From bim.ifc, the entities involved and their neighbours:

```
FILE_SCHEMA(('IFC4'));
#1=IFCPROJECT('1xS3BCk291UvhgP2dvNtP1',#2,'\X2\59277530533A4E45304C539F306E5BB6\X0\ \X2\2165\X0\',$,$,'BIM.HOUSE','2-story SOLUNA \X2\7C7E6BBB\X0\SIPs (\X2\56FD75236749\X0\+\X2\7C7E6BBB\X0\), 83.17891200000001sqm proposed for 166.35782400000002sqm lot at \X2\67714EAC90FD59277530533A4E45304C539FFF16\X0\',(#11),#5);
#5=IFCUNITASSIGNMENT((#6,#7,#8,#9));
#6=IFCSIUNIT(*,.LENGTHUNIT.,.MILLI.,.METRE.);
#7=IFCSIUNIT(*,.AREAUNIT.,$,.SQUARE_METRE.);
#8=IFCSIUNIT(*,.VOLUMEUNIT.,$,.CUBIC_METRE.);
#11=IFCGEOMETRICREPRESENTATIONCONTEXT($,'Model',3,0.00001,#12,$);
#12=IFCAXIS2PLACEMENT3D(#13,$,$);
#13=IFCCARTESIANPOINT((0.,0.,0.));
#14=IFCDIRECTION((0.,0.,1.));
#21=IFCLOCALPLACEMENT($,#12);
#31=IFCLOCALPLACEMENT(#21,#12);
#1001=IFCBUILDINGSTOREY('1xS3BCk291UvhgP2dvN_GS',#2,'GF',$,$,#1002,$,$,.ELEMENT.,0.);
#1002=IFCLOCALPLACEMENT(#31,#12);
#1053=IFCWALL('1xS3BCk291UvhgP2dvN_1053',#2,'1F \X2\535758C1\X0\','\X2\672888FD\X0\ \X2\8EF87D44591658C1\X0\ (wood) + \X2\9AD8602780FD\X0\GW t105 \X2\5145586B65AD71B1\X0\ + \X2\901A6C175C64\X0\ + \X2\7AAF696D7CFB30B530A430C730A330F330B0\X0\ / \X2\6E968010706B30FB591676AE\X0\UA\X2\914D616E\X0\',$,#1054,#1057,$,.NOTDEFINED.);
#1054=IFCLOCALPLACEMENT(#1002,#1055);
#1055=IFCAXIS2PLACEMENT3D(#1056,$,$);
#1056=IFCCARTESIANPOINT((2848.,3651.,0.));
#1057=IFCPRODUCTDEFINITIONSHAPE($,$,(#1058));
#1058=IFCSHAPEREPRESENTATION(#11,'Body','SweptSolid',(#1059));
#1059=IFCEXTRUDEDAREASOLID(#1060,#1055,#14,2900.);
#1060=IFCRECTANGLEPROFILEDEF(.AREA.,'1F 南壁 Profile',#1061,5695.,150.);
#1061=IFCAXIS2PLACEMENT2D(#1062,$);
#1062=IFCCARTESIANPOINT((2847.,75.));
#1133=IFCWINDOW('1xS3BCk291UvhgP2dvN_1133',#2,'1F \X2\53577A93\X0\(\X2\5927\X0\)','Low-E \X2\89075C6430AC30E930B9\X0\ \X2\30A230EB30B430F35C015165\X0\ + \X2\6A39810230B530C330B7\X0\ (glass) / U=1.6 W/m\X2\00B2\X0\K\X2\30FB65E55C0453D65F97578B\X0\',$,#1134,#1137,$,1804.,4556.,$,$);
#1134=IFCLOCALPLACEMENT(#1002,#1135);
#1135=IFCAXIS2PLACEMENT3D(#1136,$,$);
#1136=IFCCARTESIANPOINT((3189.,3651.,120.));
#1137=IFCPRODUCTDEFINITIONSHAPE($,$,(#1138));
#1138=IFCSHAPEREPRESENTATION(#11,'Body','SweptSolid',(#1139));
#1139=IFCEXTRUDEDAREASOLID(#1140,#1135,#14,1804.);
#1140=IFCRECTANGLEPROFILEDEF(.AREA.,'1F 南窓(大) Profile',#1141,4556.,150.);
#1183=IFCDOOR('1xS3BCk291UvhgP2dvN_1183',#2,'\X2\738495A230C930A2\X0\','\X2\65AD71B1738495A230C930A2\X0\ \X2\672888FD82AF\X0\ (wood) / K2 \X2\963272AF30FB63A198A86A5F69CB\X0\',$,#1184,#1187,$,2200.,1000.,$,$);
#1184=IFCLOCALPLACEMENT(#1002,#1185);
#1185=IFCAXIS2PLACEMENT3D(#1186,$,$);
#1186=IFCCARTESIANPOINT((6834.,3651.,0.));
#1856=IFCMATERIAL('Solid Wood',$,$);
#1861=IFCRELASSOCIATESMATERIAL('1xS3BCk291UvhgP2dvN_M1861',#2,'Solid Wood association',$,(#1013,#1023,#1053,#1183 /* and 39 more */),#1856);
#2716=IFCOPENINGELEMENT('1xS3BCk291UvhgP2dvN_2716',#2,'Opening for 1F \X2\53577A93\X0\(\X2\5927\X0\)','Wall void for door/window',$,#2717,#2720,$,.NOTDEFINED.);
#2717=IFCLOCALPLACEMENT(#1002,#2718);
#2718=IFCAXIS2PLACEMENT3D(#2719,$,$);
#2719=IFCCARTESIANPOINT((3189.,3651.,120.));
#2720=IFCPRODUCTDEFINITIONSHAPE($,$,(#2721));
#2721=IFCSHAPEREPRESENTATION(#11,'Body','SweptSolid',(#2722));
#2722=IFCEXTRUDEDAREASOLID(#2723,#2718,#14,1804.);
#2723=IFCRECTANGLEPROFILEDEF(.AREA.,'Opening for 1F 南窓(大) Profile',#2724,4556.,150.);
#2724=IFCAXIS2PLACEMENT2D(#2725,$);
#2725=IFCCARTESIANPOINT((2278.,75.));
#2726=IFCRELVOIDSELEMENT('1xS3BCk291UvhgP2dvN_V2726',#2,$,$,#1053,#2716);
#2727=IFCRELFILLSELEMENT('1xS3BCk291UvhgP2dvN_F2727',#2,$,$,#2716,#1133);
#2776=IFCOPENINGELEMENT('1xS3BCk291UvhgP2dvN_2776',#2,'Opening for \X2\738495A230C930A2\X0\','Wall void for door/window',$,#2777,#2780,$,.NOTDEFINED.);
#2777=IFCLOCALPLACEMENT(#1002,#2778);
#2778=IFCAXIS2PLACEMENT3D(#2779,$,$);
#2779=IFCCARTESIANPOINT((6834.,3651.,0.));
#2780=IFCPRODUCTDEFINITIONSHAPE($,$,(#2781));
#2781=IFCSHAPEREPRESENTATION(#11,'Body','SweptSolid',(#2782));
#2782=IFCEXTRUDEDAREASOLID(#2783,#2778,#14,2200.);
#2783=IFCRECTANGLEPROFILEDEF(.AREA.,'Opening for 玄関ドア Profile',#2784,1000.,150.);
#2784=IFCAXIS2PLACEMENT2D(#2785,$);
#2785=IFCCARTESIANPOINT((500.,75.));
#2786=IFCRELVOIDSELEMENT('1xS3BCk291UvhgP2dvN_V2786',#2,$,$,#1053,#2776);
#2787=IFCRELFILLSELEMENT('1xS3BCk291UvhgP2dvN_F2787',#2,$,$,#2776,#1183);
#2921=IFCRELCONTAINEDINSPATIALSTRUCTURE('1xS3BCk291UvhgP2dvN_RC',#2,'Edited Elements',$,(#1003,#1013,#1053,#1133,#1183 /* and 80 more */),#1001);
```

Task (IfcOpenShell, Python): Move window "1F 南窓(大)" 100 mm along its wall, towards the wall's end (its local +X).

```python
import ifcopenshell
import ifcopenshell.api.geometry
import ifcopenshell.util.placement

model = ifcopenshell.open("bim.ifc")

window = model.by_guid("1xS3BCk291UvhgP2dvN_1133")
opening = window.FillsVoids[0].RelatingOpeningElement
wall = opening.VoidsElements[0].RelatingBuildingElement

wall_matrix = ifcopenshell.util.placement.get_local_placement(wall.ObjectPlacement)
shift = wall_matrix[:3, 0] * 100.0
before = ifcopenshell.util.placement.get_local_placement(window.ObjectPlacement)[:3, 3].copy()

# The window is not placed relative to its opening, so move both.
for product in (opening, window):
    matrix = ifcopenshell.util.placement.get_local_placement(product.ObjectPlacement)
    matrix[:3, 3] += shift
    ifcopenshell.api.geometry.edit_object_placement(model, product=product, matrix=matrix, is_si=False)

after = ifcopenshell.util.placement.get_local_placement(window.ObjectPlacement)[:3, 3]
print("window moved by", (after - before).round(3) + 0.0)

model.write("bim_rev.ifc")
```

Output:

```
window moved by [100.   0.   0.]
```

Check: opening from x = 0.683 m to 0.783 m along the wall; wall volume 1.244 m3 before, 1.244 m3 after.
